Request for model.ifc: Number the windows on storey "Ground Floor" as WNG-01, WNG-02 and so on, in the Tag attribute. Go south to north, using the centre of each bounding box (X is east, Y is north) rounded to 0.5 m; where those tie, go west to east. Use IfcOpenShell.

First a look at what the model holds.

```python
import ifcopenshell
import ifcopenshell.util.element
import ifcopenshell.util.placement

model = ifcopenshell.open("model.ifc")
print(model.schema)
storey = next(s for s in model.by_type("IfcBuildingStorey") if s.Name == "Ground Floor")
windows = [e for e in ifcopenshell.util.element.get_decomposition(storey) if e.is_a("IfcWindow")]
for e in sorted(windows, key=lambda e: e.id()):
    origin = ifcopenshell.util.placement.get_local_placement(e.ObjectPlacement)[:3, 3]
    print(e.id(), e.Tag, e.Name, origin.round(2) + 0.0, sep=" | ")
```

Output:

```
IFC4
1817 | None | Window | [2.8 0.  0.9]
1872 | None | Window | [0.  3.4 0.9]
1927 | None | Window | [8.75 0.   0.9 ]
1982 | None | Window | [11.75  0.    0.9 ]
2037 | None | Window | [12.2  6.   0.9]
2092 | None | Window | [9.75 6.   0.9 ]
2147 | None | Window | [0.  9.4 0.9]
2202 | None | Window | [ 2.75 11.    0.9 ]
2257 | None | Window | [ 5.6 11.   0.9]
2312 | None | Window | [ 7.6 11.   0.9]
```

```python
import ifcopenshell
import ifcopenshell.geom
import ifcopenshell.util.element
import ifcopenshell.util.shape

model = ifcopenshell.open("model.ifc")
settings = ifcopenshell.geom.settings()
settings.set("use-world-coords", True)


def centre(element):
    shape = ifcopenshell.geom.create_shape(settings, element)
    return ifcopenshell.util.shape.get_bbox_centroid(shape.geometry)


storey = next(s for s in model.by_type("IfcBuildingStorey") if s.Name == "Ground Floor")
windows = [e for e in ifcopenshell.util.element.get_decomposition(storey) if e.is_a("IfcWindow")]

# Insertion points can sit at a corner or the storey origin, so sort by the geometry (in metres).
centres = {e: centre(e) for e in windows}
windows.sort(key=lambda e: (round(centres[e][1] / 0.5), centres[e][0]))

for i, e in enumerate(windows, start=1):
    number = f"WNG-{i:02d}"
    e.Tag = number
    print(e.id(), number)

model.write("model_v2.ifc")
```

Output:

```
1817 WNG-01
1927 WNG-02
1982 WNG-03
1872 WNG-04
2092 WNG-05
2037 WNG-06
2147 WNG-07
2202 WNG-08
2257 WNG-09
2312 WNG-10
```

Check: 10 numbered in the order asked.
